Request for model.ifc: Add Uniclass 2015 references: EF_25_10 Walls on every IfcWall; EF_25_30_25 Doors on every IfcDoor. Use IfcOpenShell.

First a look at what the model holds.

```python
import ifcopenshell

model = ifcopenshell.open("model.ifc")
print(model.schema)
print("classifications:", [c.Name for c in model.by_type("IfcClassification")])
for ifc_class in ("IfcDoor", "IfcRoof", "IfcStair", "IfcWall", "IfcWindow"):
    print(ifc_class, len(model.by_type(ifc_class)))
```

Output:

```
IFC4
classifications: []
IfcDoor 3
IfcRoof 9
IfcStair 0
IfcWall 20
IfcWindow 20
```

```python
import ifcopenshell
import ifcopenshell.api.classification

model = ifcopenshell.open("model.ifc")

system = ifcopenshell.api.classification.add_classification(model, classification="Uniclass 2015")

codes = {
    "IfcWall": ("EF_25_10", "Walls"),
    "IfcDoor": ("EF_25_30_25", "Doors"),
}
for ifc_class, (code, name) in codes.items():
    products = model.by_type(ifc_class)
    ifcopenshell.api.classification.add_reference(
        model, products=products, classification=system, identification=code, name=name
    )
    print(code, len(products))

model.write("model_updated.ifc")
```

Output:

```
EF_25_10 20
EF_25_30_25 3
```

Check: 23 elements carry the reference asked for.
